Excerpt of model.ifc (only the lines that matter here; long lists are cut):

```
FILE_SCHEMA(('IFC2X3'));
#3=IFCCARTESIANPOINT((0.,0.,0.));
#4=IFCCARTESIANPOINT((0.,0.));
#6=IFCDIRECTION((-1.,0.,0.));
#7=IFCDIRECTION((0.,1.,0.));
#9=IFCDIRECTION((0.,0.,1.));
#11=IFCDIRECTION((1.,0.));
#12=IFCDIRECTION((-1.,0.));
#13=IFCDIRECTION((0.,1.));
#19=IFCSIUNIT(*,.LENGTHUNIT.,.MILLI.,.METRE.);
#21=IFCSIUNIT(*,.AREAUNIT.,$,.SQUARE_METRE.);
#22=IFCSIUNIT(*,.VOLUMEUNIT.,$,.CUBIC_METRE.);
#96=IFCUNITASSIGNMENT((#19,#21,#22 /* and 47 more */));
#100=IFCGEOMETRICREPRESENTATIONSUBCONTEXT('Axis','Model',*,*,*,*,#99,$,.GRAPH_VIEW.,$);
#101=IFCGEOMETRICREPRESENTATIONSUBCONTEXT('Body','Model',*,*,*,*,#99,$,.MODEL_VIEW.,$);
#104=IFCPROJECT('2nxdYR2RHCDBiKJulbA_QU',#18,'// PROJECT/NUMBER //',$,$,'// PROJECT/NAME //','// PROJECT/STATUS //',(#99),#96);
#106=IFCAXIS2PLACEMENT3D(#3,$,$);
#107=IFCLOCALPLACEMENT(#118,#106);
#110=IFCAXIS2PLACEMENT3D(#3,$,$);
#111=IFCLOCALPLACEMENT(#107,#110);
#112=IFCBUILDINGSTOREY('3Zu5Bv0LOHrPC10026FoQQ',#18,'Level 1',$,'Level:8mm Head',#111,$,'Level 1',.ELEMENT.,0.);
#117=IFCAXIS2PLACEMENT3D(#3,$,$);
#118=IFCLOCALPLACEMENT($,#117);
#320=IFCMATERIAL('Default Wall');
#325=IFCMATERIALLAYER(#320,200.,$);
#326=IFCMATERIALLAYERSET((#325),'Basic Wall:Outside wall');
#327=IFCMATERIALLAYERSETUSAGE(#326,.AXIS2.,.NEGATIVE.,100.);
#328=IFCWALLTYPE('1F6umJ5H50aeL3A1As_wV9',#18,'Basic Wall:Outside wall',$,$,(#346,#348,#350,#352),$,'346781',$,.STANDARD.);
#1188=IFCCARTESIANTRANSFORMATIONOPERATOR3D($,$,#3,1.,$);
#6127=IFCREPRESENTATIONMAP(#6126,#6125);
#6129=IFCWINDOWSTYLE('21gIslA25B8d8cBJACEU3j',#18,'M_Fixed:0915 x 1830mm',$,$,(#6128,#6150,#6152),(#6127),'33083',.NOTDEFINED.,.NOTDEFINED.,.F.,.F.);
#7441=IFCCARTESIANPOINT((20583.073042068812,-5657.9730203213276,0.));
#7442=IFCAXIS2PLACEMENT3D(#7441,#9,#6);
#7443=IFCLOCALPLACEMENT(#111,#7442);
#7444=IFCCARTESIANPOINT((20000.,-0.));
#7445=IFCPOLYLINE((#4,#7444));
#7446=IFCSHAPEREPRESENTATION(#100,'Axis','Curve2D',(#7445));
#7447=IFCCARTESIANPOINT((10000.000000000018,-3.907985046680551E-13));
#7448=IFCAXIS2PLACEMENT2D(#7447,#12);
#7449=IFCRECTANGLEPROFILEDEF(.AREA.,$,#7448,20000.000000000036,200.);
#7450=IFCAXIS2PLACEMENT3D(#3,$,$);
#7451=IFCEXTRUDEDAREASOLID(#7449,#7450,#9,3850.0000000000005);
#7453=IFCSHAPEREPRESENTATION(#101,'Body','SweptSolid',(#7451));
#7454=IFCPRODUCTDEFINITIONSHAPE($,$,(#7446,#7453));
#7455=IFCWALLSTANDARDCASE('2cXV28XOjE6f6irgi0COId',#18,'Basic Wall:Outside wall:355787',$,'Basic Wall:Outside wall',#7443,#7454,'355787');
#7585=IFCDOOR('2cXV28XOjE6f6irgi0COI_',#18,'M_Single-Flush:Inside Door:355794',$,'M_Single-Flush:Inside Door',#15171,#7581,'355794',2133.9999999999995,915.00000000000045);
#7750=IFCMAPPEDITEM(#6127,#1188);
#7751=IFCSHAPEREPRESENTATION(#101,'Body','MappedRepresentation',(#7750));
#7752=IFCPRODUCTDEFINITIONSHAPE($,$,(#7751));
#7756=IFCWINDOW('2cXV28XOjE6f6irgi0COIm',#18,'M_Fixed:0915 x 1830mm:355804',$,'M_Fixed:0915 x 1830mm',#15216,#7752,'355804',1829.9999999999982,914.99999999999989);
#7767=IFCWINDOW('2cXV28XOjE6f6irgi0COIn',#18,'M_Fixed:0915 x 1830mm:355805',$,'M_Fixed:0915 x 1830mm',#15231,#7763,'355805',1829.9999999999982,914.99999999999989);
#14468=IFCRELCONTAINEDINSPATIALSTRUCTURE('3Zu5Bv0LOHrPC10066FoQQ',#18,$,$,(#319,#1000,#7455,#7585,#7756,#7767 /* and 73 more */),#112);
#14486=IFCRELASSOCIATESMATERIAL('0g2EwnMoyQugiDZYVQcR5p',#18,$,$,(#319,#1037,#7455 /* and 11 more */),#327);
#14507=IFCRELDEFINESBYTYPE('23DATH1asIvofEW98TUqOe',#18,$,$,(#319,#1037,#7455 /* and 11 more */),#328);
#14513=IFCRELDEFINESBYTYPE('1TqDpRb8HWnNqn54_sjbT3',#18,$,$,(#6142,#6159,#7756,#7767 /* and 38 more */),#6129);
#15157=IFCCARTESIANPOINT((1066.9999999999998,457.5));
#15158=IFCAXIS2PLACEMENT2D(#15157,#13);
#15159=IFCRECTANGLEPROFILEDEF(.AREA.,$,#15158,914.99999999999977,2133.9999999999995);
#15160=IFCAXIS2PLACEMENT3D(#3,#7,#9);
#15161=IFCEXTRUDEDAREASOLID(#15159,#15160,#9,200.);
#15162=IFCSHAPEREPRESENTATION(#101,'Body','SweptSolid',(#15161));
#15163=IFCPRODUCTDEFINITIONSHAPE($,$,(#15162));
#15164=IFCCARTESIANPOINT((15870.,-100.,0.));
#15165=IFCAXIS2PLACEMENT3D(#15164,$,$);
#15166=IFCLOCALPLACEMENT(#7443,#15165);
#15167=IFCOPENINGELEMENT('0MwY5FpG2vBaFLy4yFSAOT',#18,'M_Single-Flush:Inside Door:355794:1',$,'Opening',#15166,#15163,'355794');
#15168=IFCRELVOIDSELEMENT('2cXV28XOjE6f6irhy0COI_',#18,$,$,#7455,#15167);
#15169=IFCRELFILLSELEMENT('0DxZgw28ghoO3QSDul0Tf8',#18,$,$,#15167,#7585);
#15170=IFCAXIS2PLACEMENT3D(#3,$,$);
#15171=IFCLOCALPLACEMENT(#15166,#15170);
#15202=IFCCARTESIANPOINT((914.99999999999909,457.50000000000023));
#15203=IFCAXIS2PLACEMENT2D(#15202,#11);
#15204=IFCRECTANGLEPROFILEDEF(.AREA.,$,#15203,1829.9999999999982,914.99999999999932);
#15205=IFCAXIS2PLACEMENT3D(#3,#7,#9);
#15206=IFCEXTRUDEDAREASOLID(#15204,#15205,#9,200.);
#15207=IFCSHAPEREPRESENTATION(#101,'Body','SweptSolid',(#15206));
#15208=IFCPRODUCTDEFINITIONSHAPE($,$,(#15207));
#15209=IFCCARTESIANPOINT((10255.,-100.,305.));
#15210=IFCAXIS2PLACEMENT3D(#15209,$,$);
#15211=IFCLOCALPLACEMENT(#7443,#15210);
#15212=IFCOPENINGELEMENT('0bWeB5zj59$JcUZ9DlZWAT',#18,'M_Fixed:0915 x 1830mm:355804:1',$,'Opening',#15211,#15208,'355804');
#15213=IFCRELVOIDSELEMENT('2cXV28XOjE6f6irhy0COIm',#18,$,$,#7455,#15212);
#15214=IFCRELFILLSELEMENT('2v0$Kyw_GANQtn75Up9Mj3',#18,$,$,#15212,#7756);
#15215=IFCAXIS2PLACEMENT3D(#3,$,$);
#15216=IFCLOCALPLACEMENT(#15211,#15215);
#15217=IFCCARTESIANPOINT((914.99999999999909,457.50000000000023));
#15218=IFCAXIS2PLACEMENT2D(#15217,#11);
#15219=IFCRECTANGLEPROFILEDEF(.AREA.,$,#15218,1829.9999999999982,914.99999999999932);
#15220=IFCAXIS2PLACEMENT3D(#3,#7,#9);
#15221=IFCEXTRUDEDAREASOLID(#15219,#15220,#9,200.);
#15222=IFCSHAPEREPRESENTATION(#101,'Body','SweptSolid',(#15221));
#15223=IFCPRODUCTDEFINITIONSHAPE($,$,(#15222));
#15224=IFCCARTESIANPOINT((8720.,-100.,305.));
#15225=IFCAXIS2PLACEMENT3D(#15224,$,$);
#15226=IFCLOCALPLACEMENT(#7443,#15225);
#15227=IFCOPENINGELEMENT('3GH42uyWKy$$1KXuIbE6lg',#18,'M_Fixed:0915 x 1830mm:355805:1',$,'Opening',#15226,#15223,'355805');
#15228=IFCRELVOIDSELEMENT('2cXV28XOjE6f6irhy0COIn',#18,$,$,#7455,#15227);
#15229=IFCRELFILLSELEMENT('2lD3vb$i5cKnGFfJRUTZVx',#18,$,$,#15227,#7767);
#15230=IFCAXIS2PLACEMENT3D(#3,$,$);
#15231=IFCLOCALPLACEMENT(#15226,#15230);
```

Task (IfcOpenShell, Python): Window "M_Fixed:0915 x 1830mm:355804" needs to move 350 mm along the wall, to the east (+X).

```python
import ifcopenshell
import ifcopenshell.api.geometry
import ifcopenshell.util.placement
import ifcopenshell.util.unit

model = ifcopenshell.open("model.ifc")
unit_scale = ifcopenshell.util.unit.calculate_unit_scale(model)

window = model.by_guid("2cXV28XOjE6f6irgi0COIm")
opening = window.FillsVoids[0].RelatingOpeningElement
wall = opening.VoidsElements[0].RelatingBuildingElement

wall_matrix = ifcopenshell.util.placement.get_local_placement(wall.ObjectPlacement)
shift = wall_matrix[:3, 0] * -0.35 / unit_scale
before = ifcopenshell.util.placement.get_local_placement(window.ObjectPlacement)[:3, 3].copy()

# The window is placed relative to its opening, so it follows when the opening moves.
matrix = ifcopenshell.util.placement.get_local_placement(opening.ObjectPlacement)
matrix[:3, 3] += shift
ifcopenshell.api.geometry.edit_object_placement(
    model, product=opening, matrix=matrix, is_si=False, should_transform_children=True
)

after = ifcopenshell.util.placement.get_local_placement(window.ObjectPlacement)[:3, 3]
print("window moved by", (after - before).round(3) + 0.0)

model.write("model_updated.ifc")
```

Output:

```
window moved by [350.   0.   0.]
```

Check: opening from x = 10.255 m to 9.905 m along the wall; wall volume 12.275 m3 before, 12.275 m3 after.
